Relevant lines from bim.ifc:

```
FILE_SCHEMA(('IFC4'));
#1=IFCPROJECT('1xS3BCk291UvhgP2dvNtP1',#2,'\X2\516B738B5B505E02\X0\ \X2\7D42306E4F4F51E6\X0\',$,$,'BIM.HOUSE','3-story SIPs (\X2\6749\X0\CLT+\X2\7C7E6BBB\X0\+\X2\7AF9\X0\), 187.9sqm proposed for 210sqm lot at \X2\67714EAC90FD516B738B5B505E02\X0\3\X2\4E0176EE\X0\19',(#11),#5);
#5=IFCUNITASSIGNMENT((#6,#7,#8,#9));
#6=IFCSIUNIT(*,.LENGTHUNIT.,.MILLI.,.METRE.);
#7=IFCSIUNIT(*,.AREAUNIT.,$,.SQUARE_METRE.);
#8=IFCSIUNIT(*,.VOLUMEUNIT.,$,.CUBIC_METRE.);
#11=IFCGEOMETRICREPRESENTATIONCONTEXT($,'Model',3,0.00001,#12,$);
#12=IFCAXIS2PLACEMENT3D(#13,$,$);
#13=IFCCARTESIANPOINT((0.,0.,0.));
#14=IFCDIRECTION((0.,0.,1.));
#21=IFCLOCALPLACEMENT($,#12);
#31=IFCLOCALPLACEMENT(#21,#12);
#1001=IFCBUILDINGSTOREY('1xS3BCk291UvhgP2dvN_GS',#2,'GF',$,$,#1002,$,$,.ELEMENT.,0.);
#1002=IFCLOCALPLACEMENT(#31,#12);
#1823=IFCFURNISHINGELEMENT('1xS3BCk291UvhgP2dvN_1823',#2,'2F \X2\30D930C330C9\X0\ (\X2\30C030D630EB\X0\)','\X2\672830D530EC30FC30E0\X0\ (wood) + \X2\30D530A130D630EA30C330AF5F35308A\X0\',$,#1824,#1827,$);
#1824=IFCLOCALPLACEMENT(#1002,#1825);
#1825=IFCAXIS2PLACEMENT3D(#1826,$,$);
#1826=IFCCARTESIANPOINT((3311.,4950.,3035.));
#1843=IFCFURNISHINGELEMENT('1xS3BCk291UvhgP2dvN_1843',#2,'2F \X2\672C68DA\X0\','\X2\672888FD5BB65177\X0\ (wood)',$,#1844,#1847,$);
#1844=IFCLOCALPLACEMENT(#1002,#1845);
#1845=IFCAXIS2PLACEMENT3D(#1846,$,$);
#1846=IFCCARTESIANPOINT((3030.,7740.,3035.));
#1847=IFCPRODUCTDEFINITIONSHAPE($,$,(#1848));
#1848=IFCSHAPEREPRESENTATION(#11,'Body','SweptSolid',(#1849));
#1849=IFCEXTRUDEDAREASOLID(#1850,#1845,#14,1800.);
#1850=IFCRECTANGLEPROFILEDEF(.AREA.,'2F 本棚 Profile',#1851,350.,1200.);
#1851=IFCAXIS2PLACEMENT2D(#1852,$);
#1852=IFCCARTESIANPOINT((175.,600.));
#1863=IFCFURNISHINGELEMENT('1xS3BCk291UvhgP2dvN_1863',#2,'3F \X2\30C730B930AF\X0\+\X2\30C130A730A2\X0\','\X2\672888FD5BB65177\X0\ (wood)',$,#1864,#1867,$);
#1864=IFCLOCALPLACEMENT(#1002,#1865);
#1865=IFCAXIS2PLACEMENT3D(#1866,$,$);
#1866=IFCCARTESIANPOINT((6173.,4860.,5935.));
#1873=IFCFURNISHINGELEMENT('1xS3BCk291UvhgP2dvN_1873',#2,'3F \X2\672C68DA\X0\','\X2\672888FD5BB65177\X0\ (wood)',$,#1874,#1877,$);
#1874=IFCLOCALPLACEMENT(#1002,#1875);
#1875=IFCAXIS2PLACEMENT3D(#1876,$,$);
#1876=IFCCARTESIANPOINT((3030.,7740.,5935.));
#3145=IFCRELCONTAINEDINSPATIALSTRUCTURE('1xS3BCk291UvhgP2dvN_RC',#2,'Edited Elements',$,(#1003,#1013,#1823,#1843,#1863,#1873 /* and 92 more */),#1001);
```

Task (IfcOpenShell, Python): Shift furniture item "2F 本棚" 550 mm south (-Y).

```python
import ifcopenshell
import ifcopenshell.api.geometry
import ifcopenshell.util.placement

model = ifcopenshell.open("bim.ifc")

item = model.by_guid("1xS3BCk291UvhgP2dvN_1843")
matrix = ifcopenshell.util.placement.get_local_placement(item.ObjectPlacement)
matrix[1, 3] -= 550.0
ifcopenshell.api.geometry.edit_object_placement(model, product=item, matrix=matrix, is_si=False)

print(ifcopenshell.util.placement.get_local_placement(item.ObjectPlacement).round(3) + 0.0)

model.write("bim_edited.ifc")
```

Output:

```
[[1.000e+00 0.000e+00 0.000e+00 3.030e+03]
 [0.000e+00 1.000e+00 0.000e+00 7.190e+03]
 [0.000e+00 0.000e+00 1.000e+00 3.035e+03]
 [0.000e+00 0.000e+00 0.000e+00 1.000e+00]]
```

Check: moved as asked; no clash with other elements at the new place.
